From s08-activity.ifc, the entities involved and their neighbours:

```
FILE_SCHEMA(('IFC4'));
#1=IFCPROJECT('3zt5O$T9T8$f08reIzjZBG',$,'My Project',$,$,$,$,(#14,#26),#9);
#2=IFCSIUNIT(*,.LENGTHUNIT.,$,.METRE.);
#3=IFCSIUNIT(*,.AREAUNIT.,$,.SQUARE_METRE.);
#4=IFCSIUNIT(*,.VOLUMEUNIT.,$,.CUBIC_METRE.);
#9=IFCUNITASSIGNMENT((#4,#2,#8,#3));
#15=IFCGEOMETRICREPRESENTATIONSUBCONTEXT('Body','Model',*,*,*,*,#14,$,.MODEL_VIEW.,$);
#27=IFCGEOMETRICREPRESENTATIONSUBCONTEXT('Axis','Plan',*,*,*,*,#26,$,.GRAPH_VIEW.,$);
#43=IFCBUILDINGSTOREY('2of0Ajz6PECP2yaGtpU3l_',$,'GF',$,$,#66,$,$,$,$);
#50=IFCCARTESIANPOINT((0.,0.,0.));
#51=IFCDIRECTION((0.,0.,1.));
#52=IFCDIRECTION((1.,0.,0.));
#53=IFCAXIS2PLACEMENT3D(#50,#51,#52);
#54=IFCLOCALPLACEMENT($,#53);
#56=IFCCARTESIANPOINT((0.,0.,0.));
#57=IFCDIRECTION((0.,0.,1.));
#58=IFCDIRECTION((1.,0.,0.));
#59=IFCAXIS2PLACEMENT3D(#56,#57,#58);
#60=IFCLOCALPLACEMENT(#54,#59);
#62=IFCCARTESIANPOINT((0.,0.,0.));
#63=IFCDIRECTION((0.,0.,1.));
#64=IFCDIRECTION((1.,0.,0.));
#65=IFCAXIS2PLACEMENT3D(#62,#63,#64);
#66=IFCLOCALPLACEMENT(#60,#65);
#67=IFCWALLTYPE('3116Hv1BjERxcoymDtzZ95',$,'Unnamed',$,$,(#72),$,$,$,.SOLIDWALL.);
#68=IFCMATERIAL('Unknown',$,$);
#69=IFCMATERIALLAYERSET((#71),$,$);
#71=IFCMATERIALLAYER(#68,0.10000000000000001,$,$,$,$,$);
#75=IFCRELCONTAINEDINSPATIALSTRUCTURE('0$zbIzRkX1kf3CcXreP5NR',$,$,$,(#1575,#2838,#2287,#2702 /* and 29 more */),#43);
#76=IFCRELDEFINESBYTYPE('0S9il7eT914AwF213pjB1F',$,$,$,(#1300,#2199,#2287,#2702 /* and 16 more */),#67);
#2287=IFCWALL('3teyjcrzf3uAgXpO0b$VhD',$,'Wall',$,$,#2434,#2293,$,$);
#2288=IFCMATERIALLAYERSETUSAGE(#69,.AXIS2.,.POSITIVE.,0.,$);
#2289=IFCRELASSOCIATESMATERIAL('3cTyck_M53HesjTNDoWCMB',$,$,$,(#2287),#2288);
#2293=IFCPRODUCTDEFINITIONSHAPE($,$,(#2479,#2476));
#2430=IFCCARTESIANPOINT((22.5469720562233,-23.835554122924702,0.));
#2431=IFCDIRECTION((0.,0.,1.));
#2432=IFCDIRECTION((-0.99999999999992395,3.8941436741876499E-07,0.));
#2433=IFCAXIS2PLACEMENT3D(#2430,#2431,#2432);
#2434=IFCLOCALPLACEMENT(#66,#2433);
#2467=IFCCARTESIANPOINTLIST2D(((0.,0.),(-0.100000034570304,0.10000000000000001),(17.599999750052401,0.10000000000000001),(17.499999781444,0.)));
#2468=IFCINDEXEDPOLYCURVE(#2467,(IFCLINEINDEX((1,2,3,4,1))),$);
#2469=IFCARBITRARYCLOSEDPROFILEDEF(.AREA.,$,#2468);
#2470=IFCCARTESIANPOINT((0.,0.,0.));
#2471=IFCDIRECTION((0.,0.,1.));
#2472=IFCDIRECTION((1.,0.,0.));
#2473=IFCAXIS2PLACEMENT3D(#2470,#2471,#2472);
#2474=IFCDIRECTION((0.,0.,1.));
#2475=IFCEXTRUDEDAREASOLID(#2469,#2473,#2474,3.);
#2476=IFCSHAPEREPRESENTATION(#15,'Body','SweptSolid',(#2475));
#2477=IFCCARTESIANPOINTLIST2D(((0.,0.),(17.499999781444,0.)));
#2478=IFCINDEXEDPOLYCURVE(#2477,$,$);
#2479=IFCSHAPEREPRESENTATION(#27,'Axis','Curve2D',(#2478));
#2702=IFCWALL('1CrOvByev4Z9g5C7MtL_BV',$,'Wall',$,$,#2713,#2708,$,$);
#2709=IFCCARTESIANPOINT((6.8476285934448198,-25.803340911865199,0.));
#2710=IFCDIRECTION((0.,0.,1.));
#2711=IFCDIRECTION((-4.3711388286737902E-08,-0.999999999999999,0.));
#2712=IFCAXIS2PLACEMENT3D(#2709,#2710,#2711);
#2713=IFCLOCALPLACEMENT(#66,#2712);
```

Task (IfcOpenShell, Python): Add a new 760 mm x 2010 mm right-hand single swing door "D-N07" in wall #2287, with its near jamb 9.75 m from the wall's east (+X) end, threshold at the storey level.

```python
import numpy as np
import ifcopenshell
import ifcopenshell.api.feature
import ifcopenshell.api.geometry
import ifcopenshell.api.root
import ifcopenshell.api.spatial
import ifcopenshell.geom
import ifcopenshell.util.element
import ifcopenshell.util.placement
import ifcopenshell.util.representation
import ifcopenshell.util.shape
import ifcopenshell.util.unit

model = ifcopenshell.open("s08-activity.ifc")
unit_scale = ifcopenshell.util.unit.calculate_unit_scale(model)
settings = ifcopenshell.geom.settings()


def volume(element):
    """Net volume in cubic metres, openings subtracted."""
    shape = ifcopenshell.geom.create_shape(settings, element)
    return ifcopenshell.util.shape.get_volume(shape.geometry)


wall = model.by_id(2287)
storey = ifcopenshell.util.element.get_container(wall, ifc_class="IfcBuildingStorey")
context = ifcopenshell.util.representation.get_context(model, "Model", "Body", "MODEL_VIEW")
before = volume(wall)

width, height, from_end, sill = 0.76, 2.01, 9.75, 0.0  # metres

# The wall runs along its own X axis, and the end named is its -X end.
wall_shape = ifcopenshell.geom.create_shape(settings, wall)
x, y, z = ifcopenshell.util.shape.get_vertices(wall_shape.geometry).T
start = x.min() + from_end
face, thickness = float(y.min()), float(y.max() - y.min())
wall_matrix = ifcopenshell.util.placement.get_local_placement(wall.ObjectPlacement)
level = ifcopenshell.util.placement.get_local_placement(storey.ObjectPlacement)[2, 3]


def in_wall(x, y):
    """Placement at x, y metres in the wall's axes, at sill height."""
    matrix = wall_matrix.copy()
    matrix[:, 3] = wall_matrix @ np.array([x / unit_scale, y / unit_scale, 0.0, 1.0])
    matrix[2, 3] = level + sill / unit_scale
    return matrix


# Opening: a box that overshoots both wall faces by 50 mm.
opening = ifcopenshell.api.root.create_entity(model, ifc_class="IfcOpeningElement", predefined_type="OPENING")
box = ifcopenshell.api.geometry.add_wall_representation(
    model, context=context, length=width, height=height, thickness=thickness + 0.1
)
ifcopenshell.api.geometry.assign_representation(model, product=opening, representation=box)
ifcopenshell.api.geometry.edit_object_placement(model, product=opening, matrix=in_wall(start, face - 0.05), is_si=False)
ifcopenshell.api.feature.add_feature(model, feature=opening, element=wall)

door = ifcopenshell.api.root.create_entity(model, ifc_class="IfcDoor", name="D-N07", predefined_type="DOOR")
door.OverallWidth, door.OverallHeight = width / unit_scale, height / unit_scale
door.OperationType = "SINGLE_SWING_RIGHT"
body = ifcopenshell.api.geometry.add_door_representation(
    model,
    context=context,
    overall_width=door.OverallWidth,
    overall_height=door.OverallHeight,
    operation_type="SINGLE_SWING_RIGHT",
    lining_properties={"LiningDepth": thickness / unit_scale, "ThresholdDepth": thickness / unit_scale},
)
ifcopenshell.api.geometry.assign_representation(model, product=door, representation=body)
ifcopenshell.api.spatial.assign_container(model, products=[door], relating_structure=storey)
ifcopenshell.api.feature.add_filling(model, opening=opening, element=door)

# The lining spans the wall, so the door starts at the wall face.
ifcopenshell.api.geometry.edit_object_placement(model, product=door, matrix=in_wall(start, face), is_si=False)

after = volume(wall)

print(f"wall volume {before:.3f} -> {after:.3f} m3")

model.write("s08-activity_v2.ifc")
```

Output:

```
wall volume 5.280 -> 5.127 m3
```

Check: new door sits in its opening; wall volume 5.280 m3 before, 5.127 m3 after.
